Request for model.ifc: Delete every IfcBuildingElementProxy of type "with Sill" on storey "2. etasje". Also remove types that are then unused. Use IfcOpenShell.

First a look at what the model holds.

```python
import ifcopenshell
import ifcopenshell.util.element

model = ifcopenshell.open("model.ifc")
print(model.schema)
storey = next(s for s in model.by_type("IfcBuildingStorey") if s.Name == "2. etasje")
proxies = [e for e in ifcopenshell.util.element.get_decomposition(storey) if e.is_a("IfcBuildingElementProxy")]
seen = {}
for e in proxies:
    element_type = ifcopenshell.util.element.get_type(e)
    name = element_type.Name if element_type not in (None, e) else None
    seen[name] = seen.get(name, 0) + 1
for name, count in sorted(seen.items(), key=str):
    print(count, "x", name)
```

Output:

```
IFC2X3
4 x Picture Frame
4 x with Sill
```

```python
import ifcopenshell
import ifcopenshell.api.root
import ifcopenshell.util.element

model = ifcopenshell.open("model.ifc")

storey = next(s for s in model.by_type("IfcBuildingStorey") if s.Name == "2. etasje")
proxies = [e for e in ifcopenshell.util.element.get_decomposition(storey) if e.is_a("IfcBuildingElementProxy")]
targets = [e for e in proxies if (t := ifcopenshell.util.element.get_type(e)) not in (None, e) and t.Name == "with Sill"]
types = {ifcopenshell.util.element.get_type(e) for e in targets} - {None, *targets}

for e in targets:
    ifcopenshell.api.root.remove_product(model, product=e)
print(len(targets), "removed")

unused = [t for t in types if not ifcopenshell.util.element.get_types(t)]
for t in unused:
    ifcopenshell.api.root.remove_product(model, product=t)
print(len(unused), "unused types removed")

model.write("model_edited.ifc")
```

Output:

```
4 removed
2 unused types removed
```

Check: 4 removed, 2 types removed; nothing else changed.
